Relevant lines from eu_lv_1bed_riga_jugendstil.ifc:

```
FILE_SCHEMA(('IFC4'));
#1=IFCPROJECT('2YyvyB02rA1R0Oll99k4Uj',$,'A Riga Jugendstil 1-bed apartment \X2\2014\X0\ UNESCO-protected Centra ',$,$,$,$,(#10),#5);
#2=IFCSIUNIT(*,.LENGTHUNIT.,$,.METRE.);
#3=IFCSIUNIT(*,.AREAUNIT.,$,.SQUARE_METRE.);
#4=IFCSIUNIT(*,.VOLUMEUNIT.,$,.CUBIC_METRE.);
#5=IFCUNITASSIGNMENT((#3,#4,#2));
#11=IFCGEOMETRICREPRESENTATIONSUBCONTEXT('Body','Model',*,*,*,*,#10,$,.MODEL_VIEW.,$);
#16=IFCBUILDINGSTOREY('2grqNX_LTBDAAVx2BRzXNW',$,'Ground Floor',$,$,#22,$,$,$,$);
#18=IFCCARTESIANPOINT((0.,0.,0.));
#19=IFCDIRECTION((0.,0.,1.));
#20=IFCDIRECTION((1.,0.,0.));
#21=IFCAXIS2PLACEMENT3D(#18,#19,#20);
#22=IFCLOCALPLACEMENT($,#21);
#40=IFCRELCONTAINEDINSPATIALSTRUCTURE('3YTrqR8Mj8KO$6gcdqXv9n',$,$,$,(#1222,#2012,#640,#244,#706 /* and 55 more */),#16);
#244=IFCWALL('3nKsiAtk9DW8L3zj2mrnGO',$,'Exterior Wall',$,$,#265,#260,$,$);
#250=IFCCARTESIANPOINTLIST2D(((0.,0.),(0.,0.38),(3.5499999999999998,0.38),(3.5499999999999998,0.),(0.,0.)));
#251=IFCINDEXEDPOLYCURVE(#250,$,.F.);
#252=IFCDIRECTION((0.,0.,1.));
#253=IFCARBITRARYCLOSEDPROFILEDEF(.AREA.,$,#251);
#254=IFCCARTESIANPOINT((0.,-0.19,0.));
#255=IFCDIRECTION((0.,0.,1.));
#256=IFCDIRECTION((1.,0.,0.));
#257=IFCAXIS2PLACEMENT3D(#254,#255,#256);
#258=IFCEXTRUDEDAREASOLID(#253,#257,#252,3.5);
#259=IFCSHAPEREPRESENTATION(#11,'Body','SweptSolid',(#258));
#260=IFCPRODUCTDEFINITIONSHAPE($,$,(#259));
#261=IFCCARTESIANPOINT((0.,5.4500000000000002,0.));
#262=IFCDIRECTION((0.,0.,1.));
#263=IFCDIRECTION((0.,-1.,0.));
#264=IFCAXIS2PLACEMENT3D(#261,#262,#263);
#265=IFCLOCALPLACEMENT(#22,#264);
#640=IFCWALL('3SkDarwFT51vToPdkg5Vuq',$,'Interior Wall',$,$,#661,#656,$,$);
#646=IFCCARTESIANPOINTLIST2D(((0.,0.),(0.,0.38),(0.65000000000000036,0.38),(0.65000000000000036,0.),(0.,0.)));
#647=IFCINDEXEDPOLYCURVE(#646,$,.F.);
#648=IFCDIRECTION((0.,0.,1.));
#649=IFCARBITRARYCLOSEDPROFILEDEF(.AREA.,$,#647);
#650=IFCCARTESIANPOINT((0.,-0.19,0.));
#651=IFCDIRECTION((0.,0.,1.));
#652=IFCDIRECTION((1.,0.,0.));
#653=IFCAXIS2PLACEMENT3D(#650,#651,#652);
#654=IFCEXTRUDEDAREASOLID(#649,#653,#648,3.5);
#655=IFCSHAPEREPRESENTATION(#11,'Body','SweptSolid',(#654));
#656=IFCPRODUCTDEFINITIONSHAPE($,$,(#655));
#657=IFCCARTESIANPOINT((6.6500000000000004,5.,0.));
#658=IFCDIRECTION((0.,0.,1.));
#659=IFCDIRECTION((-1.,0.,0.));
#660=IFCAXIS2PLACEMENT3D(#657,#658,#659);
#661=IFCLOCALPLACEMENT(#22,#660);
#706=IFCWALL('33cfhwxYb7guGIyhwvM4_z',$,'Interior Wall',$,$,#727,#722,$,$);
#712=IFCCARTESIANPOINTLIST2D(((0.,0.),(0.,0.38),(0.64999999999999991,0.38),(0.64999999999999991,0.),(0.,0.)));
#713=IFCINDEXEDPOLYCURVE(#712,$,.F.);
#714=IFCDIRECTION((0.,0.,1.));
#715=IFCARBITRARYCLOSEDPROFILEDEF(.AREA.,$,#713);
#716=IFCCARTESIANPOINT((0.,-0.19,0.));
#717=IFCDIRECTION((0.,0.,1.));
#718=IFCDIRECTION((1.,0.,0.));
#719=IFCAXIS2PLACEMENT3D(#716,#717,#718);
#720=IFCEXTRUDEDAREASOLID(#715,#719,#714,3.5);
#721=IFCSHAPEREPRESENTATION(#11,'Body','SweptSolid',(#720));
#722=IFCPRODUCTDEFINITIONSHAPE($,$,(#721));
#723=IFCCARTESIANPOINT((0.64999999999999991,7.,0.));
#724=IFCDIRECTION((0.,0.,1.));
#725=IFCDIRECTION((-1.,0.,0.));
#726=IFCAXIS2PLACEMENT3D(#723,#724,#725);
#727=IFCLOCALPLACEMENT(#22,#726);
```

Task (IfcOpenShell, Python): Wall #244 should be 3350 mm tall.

```python
import ifcopenshell
import ifcopenshell.geom
import ifcopenshell.util.representation
import ifcopenshell.util.shape
import ifcopenshell.util.unit

model = ifcopenshell.open("eu_lv_1bed_riga_jugendstil.ifc")
unit_scale = ifcopenshell.util.unit.calculate_unit_scale(model)
settings = ifcopenshell.geom.settings()


def volume(element):
    """Net volume in cubic metres, openings subtracted."""
    shape = ifcopenshell.geom.create_shape(settings, element)
    return ifcopenshell.util.shape.get_volume(shape.geometry)


wall = model.by_guid("3nKsiAtk9DW8L3zj2mrnGO")
before = volume(wall)

body = ifcopenshell.util.representation.get_representation(wall, "Model", "Body")
solid = body.Items[0]
old_height = solid.Depth
solid.Depth = 3.35 / unit_scale
after = volume(wall)

print(f"height {old_height:g} -> {solid.Depth:g}, volume {before:.3f} -> {after:.3f} m3")

model.write("eu_lv_1bed_riga_jugendstil-out.ifc")
```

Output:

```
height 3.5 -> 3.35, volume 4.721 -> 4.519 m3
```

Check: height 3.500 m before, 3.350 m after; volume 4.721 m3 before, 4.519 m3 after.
